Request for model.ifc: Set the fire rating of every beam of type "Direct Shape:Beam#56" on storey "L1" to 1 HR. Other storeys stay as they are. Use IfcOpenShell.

First a look at what the model holds.

```python
import ifcopenshell
import ifcopenshell.util.element

model = ifcopenshell.open("model.ifc")
print(model.schema)
storey = next(s for s in model.by_type("IfcBuildingStorey") if s.Name == "L1")
beams = [e for e in ifcopenshell.util.element.get_decomposition(storey) if e.is_a("IfcBeam")]
seen = {}
for e in beams:
    element_type = ifcopenshell.util.element.get_type(e)
    key = (element_type.Name if element_type != e and element_type else None, ifcopenshell.util.element.get_pset(e, "Pset_BeamCommon", "FireRating"))
    seen[key] = seen.get(key, 0) + 1
for (name, value), count in sorted(seen.items(), key=str):
    print(count, "x", name, "|", value)
```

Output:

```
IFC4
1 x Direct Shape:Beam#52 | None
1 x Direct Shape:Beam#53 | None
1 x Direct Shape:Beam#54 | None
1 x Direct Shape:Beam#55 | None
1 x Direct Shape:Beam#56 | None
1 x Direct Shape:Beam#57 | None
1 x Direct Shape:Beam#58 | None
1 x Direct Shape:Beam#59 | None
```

```python
import ifcopenshell
import ifcopenshell.api.pset
import ifcopenshell.util.element

model = ifcopenshell.open("model.ifc")

storey = next(s for s in model.by_type("IfcBuildingStorey") if s.Name == "L1")
beams = [e for e in ifcopenshell.util.element.get_decomposition(storey) if e.is_a("IfcBeam")]

count = 0
for e in beams:
    element_type = ifcopenshell.util.element.get_type(e)
    if element_type in (None, e) or element_type.Name != "Direct Shape:Beam#56":
        continue
    # add_pset returns the element's existing set when there is one.
    pset = ifcopenshell.api.pset.add_pset(model, product=e, name="Pset_BeamCommon")
    ifcopenshell.api.pset.edit_pset(model, pset=pset, properties={"FireRating": "1 HR"})
    count += 1

print(count, "beams updated")

model.write("model_updated.ifc")
```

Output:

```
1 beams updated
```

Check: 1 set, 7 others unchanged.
